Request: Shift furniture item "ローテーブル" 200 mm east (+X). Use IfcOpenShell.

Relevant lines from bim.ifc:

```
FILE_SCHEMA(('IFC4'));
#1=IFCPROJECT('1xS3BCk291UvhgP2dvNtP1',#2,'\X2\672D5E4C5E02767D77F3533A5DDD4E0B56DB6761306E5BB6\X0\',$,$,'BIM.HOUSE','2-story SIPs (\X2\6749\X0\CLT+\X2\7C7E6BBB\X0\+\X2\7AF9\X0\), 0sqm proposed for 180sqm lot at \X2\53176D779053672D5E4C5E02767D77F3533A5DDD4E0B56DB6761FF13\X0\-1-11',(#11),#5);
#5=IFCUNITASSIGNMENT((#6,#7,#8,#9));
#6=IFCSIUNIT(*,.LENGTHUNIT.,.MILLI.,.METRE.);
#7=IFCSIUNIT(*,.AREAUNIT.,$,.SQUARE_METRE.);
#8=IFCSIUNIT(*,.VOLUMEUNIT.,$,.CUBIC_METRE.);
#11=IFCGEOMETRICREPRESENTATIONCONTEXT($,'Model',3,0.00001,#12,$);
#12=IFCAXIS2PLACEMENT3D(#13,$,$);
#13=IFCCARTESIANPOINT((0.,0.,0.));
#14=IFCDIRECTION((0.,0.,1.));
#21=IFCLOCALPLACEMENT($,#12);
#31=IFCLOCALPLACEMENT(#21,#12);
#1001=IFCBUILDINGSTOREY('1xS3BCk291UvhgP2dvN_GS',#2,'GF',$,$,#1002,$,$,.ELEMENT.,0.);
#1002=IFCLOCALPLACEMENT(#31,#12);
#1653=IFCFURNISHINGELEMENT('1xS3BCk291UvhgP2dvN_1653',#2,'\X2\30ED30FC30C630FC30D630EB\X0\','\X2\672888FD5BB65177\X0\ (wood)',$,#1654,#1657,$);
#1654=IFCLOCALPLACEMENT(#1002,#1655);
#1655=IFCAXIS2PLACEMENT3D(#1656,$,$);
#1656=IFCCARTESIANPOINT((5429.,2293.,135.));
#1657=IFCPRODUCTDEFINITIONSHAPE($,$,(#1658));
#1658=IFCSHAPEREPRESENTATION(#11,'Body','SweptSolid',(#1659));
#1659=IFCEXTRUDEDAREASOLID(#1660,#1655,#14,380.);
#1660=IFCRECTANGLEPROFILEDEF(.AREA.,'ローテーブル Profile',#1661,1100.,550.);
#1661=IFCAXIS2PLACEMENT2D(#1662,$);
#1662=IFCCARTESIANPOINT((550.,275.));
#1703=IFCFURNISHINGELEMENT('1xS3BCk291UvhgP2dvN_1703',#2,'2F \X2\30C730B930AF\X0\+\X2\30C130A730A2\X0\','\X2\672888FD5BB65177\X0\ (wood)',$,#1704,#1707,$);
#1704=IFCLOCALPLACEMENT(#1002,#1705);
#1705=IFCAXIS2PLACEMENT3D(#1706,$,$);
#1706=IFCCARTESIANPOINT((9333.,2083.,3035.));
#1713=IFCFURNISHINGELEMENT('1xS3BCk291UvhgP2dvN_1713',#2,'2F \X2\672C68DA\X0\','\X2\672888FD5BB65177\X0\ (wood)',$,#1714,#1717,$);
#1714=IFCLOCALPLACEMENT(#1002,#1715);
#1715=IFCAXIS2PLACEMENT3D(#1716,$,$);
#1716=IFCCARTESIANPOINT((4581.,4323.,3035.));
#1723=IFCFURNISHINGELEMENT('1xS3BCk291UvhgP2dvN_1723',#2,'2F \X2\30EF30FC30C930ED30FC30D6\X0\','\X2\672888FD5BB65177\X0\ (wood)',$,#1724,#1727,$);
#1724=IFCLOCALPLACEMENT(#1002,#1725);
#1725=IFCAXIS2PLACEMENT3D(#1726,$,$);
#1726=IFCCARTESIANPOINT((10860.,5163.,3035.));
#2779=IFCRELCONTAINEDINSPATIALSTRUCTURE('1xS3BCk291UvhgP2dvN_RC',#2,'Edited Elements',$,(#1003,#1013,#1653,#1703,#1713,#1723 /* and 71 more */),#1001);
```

```python
import ifcopenshell
import ifcopenshell.api.geometry
import ifcopenshell.util.placement
import ifcopenshell.util.unit

model = ifcopenshell.open("bim.ifc")
unit_scale = ifcopenshell.util.unit.calculate_unit_scale(model)

item = model.by_guid("1xS3BCk291UvhgP2dvN_1653")
matrix = ifcopenshell.util.placement.get_local_placement(item.ObjectPlacement)
matrix[0, 3] += 0.2 / unit_scale
ifcopenshell.api.geometry.edit_object_placement(model, product=item, matrix=matrix, is_si=False)

print(ifcopenshell.util.placement.get_local_placement(item.ObjectPlacement).round(3) + 0.0)

model.write("bim_v2.ifc")
```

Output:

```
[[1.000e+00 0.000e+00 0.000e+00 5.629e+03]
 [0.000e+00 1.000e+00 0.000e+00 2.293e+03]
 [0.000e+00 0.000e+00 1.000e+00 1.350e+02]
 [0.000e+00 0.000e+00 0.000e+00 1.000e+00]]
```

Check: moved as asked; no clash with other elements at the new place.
